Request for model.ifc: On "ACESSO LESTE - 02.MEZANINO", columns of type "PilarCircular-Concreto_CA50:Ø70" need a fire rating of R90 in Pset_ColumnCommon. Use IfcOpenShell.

First a look at what the model holds.

```python
import ifcopenshell
import ifcopenshell.util.element

model = ifcopenshell.open("model.ifc")
print(model.schema)
storey = next(s for s in model.by_type("IfcBuildingStorey") if s.Name == "ACESSO LESTE - 02.MEZANINO")
columns = [e for e in ifcopenshell.util.element.get_decomposition(storey) if e.is_a("IfcColumn")]
seen = {}
for e in columns:
    element_type = ifcopenshell.util.element.get_type(e)
    key = (element_type.Name if element_type != e and element_type else None, ifcopenshell.util.element.get_pset(e, "Pset_ColumnCommon", "FireRating"))
    seen[key] = seen.get(key, 0) + 1
for (name, value), count in sorted(seen.items(), key=str):
    print(count, "x", name, "|", value)
```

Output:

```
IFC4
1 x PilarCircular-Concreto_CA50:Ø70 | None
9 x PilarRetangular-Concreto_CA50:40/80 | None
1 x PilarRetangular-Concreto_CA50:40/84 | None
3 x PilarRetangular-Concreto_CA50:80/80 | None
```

```python
import ifcopenshell
import ifcopenshell.api.pset
import ifcopenshell.util.element

model = ifcopenshell.open("model.ifc")

storey = next(s for s in model.by_type("IfcBuildingStorey") if s.Name == "ACESSO LESTE - 02.MEZANINO")
columns = [e for e in ifcopenshell.util.element.get_decomposition(storey) if e.is_a("IfcColumn")]

count = 0
for e in columns:
    element_type = ifcopenshell.util.element.get_type(e)
    if element_type in (None, e) or element_type.Name != "PilarCircular-Concreto_CA50:Ø70":
        continue
    # add_pset returns the element's existing set when there is one.
    pset = ifcopenshell.api.pset.add_pset(model, product=e, name="Pset_ColumnCommon")
    ifcopenshell.api.pset.edit_pset(model, pset=pset, properties={"FireRating": "R90"})
    count += 1

print(count, "columns updated")

model.write("model_v2.ifc")
```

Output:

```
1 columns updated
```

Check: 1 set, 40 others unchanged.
